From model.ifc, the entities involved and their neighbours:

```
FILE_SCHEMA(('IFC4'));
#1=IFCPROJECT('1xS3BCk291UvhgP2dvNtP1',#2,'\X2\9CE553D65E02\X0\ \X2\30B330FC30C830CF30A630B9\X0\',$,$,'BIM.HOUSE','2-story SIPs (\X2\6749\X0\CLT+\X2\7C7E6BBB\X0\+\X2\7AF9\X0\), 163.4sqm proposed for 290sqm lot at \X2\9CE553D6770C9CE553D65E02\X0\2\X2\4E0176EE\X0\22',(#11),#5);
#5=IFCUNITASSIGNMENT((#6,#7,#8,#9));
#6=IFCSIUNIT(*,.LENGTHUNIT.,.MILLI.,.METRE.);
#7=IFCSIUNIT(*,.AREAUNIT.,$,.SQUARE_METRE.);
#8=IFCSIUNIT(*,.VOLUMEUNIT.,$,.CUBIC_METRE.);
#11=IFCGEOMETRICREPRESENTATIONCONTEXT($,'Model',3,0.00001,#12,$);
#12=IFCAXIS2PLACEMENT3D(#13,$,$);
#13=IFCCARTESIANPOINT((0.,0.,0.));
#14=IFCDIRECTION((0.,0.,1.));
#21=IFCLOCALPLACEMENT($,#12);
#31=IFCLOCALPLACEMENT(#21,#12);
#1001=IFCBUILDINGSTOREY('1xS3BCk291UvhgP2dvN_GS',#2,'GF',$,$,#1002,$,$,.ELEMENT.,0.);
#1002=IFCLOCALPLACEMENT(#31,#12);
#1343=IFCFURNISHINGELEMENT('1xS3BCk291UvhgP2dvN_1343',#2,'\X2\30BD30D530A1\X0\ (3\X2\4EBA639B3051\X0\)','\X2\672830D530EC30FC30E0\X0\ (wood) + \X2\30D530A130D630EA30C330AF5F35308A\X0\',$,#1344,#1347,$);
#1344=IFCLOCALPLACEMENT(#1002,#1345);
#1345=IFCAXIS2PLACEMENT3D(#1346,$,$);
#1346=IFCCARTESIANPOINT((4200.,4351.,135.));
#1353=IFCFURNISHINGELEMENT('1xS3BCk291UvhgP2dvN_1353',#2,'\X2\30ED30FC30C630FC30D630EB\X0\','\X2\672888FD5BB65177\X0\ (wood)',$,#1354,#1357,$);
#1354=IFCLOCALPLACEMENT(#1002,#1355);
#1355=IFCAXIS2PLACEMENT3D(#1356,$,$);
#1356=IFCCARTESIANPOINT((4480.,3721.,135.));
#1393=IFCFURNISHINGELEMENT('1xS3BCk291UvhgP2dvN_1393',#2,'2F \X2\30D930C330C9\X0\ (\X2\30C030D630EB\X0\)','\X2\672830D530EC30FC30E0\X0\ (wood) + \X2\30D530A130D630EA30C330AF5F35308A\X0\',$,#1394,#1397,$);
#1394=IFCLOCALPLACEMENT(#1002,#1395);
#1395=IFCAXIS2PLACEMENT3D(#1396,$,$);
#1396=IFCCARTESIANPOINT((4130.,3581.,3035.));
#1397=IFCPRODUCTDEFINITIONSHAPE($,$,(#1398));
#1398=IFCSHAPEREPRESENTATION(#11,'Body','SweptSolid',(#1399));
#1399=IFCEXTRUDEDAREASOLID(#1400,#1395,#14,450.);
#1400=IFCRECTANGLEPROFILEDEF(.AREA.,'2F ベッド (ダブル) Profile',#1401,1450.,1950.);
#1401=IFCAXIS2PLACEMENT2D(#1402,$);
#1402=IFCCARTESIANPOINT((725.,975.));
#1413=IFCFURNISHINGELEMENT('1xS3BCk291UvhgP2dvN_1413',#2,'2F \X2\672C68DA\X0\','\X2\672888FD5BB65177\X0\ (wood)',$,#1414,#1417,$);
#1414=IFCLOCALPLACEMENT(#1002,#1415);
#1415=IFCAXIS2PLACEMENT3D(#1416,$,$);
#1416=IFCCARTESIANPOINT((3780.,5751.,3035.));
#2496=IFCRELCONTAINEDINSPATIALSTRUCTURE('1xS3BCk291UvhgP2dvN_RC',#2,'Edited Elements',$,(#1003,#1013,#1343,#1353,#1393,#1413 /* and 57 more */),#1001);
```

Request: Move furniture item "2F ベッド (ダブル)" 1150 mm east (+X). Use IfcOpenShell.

```python
import ifcopenshell
import ifcopenshell.api.geometry
import ifcopenshell.util.placement
import ifcopenshell.util.unit

model = ifcopenshell.open("model.ifc")
unit_scale = ifcopenshell.util.unit.calculate_unit_scale(model)

item = model.by_id(1393)
matrix = ifcopenshell.util.placement.get_local_placement(item.ObjectPlacement)
matrix[0, 3] += 1.15 / unit_scale
ifcopenshell.api.geometry.edit_object_placement(model, product=item, matrix=matrix, is_si=False)

print(ifcopenshell.util.placement.get_local_placement(item.ObjectPlacement).round(3) + 0.0)

model.write("model_rev.ifc")
```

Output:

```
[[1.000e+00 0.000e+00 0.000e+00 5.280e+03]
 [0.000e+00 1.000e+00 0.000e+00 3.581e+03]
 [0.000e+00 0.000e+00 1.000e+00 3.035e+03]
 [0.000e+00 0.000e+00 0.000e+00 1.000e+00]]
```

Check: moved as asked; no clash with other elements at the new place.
